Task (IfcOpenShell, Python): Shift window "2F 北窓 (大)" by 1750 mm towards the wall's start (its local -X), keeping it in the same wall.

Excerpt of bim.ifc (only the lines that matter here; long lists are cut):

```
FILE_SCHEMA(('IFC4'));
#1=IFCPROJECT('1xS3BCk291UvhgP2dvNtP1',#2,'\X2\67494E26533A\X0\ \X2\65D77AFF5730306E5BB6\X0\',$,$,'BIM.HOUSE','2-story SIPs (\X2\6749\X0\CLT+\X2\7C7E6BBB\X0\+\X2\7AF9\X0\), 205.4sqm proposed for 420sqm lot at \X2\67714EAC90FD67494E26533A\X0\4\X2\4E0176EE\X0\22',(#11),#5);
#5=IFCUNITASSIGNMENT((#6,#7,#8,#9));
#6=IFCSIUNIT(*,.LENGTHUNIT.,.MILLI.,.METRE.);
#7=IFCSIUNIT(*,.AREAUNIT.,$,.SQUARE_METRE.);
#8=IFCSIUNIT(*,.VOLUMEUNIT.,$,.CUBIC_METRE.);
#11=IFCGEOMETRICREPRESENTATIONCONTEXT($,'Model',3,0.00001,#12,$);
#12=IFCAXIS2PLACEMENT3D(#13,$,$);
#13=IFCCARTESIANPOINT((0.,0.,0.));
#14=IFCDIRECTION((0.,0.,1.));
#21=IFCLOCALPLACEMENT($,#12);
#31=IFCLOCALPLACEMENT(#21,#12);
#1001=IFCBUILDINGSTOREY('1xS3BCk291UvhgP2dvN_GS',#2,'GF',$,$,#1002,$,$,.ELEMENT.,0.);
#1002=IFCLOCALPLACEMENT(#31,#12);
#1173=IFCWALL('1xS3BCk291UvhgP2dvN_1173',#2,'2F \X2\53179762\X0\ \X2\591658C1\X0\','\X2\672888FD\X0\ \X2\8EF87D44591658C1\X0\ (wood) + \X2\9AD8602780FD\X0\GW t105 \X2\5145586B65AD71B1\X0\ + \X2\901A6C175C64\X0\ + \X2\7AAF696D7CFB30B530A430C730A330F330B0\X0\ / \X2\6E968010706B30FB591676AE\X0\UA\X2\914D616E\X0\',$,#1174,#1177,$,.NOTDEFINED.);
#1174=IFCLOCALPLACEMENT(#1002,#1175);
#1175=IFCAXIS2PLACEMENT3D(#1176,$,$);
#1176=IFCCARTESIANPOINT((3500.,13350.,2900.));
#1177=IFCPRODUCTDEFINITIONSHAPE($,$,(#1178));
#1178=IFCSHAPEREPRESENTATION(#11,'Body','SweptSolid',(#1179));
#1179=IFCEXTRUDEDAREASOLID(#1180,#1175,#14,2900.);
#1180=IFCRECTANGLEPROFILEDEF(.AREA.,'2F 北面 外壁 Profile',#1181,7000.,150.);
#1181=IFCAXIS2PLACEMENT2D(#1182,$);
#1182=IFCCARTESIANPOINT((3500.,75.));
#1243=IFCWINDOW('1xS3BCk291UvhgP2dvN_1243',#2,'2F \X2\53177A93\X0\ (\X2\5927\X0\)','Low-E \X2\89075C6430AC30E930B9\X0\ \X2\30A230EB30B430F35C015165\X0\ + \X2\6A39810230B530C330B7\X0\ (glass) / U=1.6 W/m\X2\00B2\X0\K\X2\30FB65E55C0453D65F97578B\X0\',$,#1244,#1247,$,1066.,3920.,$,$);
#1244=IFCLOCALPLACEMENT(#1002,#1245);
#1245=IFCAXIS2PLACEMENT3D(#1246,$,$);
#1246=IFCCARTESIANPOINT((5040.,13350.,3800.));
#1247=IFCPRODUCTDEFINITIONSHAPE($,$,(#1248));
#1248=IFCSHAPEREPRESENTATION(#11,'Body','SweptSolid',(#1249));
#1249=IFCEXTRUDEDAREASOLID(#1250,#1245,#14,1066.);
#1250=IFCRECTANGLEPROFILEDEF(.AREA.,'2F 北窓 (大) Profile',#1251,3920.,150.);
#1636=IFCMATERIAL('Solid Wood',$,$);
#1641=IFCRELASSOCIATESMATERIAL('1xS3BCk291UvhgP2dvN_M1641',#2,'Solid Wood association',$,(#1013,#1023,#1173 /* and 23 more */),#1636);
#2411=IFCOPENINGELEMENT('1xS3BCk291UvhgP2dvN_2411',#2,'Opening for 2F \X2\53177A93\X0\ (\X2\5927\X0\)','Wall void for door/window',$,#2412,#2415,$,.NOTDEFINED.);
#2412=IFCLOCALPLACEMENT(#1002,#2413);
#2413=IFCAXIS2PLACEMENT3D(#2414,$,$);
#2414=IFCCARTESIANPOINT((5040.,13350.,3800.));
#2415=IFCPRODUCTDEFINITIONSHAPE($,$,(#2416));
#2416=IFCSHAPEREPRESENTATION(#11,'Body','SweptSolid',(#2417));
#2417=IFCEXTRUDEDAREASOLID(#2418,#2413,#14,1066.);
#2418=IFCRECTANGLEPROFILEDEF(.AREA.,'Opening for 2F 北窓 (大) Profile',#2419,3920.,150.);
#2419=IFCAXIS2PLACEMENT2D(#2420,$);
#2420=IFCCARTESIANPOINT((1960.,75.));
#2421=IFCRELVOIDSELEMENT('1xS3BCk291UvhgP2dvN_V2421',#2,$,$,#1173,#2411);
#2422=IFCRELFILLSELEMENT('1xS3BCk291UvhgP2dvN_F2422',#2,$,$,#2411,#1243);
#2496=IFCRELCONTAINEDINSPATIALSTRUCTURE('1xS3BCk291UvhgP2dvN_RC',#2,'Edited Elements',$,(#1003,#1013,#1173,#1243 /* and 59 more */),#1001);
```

```python
import ifcopenshell
import ifcopenshell.api.geometry
import ifcopenshell.util.placement
import ifcopenshell.util.unit

model = ifcopenshell.open("bim.ifc")
unit_scale = ifcopenshell.util.unit.calculate_unit_scale(model)

window = model.by_guid("1xS3BCk291UvhgP2dvN_1243")
opening = window.FillsVoids[0].RelatingOpeningElement
wall = opening.VoidsElements[0].RelatingBuildingElement

wall_matrix = ifcopenshell.util.placement.get_local_placement(wall.ObjectPlacement)
shift = wall_matrix[:3, 0] * -1.75 / unit_scale
before = ifcopenshell.util.placement.get_local_placement(window.ObjectPlacement)[:3, 3].copy()

# The window is not placed relative to its opening, so move both.
for product in (opening, window):
    matrix = ifcopenshell.util.placement.get_local_placement(product.ObjectPlacement)
    matrix[:3, 3] += shift
    ifcopenshell.api.geometry.edit_object_placement(model, product=product, matrix=matrix, is_si=False)

after = ifcopenshell.util.placement.get_local_placement(window.ObjectPlacement)[:3, 3]
print("window moved by", (after - before).round(3) + 0.0)

model.write("bim-out.ifc")
```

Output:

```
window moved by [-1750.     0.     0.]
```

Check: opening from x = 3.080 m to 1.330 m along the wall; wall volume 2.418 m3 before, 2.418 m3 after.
